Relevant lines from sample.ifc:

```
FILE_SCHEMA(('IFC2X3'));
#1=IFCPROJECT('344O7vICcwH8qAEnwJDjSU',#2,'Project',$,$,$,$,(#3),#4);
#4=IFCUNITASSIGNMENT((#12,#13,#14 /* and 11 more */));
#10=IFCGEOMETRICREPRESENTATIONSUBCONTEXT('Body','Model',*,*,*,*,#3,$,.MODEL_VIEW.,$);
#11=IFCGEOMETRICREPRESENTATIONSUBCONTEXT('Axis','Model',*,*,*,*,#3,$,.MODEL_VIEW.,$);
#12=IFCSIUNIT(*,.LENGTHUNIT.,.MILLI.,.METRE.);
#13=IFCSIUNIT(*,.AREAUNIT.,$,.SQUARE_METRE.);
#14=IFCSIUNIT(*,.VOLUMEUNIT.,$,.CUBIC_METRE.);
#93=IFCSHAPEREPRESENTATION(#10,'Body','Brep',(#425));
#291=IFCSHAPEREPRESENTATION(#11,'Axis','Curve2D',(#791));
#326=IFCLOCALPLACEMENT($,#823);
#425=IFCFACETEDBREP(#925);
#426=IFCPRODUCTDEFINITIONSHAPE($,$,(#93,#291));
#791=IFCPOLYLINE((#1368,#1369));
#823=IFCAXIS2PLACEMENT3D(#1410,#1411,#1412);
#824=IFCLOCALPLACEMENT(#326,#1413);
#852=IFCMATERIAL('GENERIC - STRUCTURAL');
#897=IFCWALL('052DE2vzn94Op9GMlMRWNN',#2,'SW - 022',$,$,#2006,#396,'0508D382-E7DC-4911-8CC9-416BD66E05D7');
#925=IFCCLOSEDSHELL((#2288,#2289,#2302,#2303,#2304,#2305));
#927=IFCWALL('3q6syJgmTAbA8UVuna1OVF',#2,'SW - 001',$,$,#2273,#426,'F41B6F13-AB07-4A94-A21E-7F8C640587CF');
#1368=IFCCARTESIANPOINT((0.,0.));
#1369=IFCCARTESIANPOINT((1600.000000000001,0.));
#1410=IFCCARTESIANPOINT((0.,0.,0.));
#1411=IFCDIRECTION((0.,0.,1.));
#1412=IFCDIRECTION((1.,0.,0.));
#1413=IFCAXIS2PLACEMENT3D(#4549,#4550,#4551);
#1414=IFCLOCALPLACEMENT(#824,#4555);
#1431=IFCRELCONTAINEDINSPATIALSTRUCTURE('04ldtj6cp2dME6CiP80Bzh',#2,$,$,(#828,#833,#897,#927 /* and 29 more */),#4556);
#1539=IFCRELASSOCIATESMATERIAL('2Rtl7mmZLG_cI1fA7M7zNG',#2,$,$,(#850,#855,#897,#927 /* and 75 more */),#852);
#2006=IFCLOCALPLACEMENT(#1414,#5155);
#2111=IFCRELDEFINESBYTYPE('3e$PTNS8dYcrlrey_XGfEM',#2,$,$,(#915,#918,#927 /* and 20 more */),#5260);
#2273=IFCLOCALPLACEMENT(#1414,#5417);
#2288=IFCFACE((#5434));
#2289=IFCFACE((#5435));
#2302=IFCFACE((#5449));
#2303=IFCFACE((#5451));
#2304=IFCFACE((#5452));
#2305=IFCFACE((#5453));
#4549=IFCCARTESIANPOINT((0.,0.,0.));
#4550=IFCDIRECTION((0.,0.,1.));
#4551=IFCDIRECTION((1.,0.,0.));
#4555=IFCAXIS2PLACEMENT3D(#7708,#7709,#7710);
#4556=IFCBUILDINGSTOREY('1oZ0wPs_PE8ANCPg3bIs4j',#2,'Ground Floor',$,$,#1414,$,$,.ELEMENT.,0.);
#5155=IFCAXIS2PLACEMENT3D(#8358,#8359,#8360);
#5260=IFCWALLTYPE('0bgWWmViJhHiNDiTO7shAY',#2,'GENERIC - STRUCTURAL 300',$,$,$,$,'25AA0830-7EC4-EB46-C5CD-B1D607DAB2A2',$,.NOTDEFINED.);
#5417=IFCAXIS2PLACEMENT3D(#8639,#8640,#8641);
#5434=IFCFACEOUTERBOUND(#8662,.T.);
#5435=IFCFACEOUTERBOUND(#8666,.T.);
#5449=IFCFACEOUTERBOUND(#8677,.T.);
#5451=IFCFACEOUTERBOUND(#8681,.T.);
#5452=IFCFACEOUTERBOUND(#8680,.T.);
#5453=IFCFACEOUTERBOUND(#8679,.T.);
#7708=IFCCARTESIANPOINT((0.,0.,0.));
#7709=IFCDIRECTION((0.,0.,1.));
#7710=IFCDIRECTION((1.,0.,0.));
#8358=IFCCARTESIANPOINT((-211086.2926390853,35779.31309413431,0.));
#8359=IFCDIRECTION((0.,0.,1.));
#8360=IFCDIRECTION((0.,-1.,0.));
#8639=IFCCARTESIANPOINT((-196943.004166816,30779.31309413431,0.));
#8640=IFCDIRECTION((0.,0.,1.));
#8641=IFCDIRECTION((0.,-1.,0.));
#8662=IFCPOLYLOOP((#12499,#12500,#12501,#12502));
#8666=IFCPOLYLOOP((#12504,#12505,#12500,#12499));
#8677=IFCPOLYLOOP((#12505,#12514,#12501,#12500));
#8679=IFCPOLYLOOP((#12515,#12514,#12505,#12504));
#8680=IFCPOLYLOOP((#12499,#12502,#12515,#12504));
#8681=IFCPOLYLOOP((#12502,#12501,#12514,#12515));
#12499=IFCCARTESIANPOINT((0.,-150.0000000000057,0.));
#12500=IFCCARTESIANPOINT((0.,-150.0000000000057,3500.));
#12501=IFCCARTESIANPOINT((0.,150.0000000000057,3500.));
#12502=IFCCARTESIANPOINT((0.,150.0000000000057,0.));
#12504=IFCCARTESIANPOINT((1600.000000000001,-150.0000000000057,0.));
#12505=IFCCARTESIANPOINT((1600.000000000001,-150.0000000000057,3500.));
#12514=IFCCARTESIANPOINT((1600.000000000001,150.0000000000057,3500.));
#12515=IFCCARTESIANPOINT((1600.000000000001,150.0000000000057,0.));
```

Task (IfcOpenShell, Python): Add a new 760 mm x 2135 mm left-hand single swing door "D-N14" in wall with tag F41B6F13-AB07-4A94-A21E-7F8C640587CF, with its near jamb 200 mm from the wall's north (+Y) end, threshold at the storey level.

```python
import numpy as np
import ifcopenshell
import ifcopenshell.api.feature
import ifcopenshell.api.geometry
import ifcopenshell.api.root
import ifcopenshell.api.spatial
import ifcopenshell.api.type
import ifcopenshell.geom
import ifcopenshell.util.element
import ifcopenshell.util.placement
import ifcopenshell.util.representation
import ifcopenshell.util.shape
import ifcopenshell.util.unit

model = ifcopenshell.open("sample.ifc")
unit_scale = ifcopenshell.util.unit.calculate_unit_scale(model)
settings = ifcopenshell.geom.settings()


def volume(element):
    """Net volume in cubic metres, openings subtracted."""
    shape = ifcopenshell.geom.create_shape(settings, element)
    return ifcopenshell.util.shape.get_volume(shape.geometry)


wall = model.by_guid("3q6syJgmTAbA8UVuna1OVF")
storey = ifcopenshell.util.element.get_container(wall, ifc_class="IfcBuildingStorey")
context = ifcopenshell.util.representation.get_context(model, "Model", "Body", "MODEL_VIEW")
before = volume(wall)

width, height, from_end, sill = 0.76, 2.135, 0.2, 0.0  # metres

# The wall runs along its own X axis, and the end named is its -X end.
wall_shape = ifcopenshell.geom.create_shape(settings, wall)
x, y, z = ifcopenshell.util.shape.get_vertices(wall_shape.geometry).T
start = x.min() + from_end
face, thickness = float(y.min()), float(y.max() - y.min())
wall_matrix = ifcopenshell.util.placement.get_local_placement(wall.ObjectPlacement)
level = ifcopenshell.util.placement.get_local_placement(storey.ObjectPlacement)[2, 3]


def in_wall(x, y):
    """Placement at x, y metres in the wall's axes, at sill height."""
    matrix = wall_matrix.copy()
    matrix[:, 3] = wall_matrix @ np.array([x / unit_scale, y / unit_scale, 0.0, 1.0])
    matrix[2, 3] = level + sill / unit_scale
    return matrix


# Opening: a box that overshoots both wall faces by 50 mm.
opening = ifcopenshell.api.root.create_entity(model, ifc_class="IfcOpeningElement")
box = ifcopenshell.api.geometry.add_wall_representation(
    model, context=context, length=width, height=height, thickness=thickness + 0.1
)
ifcopenshell.api.geometry.assign_representation(model, product=opening, representation=box)
ifcopenshell.api.geometry.edit_object_placement(model, product=opening, matrix=in_wall(start, face - 0.05), is_si=False)
ifcopenshell.api.feature.add_feature(model, feature=opening, element=wall)

door = ifcopenshell.api.root.create_entity(model, ifc_class="IfcDoor", name="D-N14")
door.OverallWidth, door.OverallHeight = width / unit_scale, height / unit_scale
body = ifcopenshell.api.geometry.add_door_representation(
    model,
    context=context,
    overall_width=door.OverallWidth,
    overall_height=door.OverallHeight,
    operation_type="SINGLE_SWING_LEFT",
    lining_properties={"LiningDepth": thickness / unit_scale, "ThresholdDepth": thickness / unit_scale},
)
ifcopenshell.api.geometry.assign_representation(model, product=door, representation=body)
ifcopenshell.api.spatial.assign_container(model, products=[door], relating_structure=storey)
fills = ifcopenshell.api.feature.add_filling(model, opening=opening, element=door)
fills.OwnerHistory = door.OwnerHistory  # required in IFC2X3

# IFC2X3 keeps the operation on the door style.
style = ifcopenshell.api.root.create_entity(model, ifc_class="IfcDoorStyle", name="D-N14")
style.OperationType, style.ConstructionType = "SINGLE_SWING_LEFT", "NOTDEFINED"
style.ParameterTakesPrecedence = style.Sizeable = False
ifcopenshell.api.type.assign_type(model, related_objects=[door], relating_type=style)

# The lining spans the wall, so the door starts at the wall face.
ifcopenshell.api.geometry.edit_object_placement(model, product=door, matrix=in_wall(start, face), is_si=False)

after = volume(wall)

print(f"wall volume {before:.3f} -> {after:.3f} m3")

model.write("sample_updated.ifc")
```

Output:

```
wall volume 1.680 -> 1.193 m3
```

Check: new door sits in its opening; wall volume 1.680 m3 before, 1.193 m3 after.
